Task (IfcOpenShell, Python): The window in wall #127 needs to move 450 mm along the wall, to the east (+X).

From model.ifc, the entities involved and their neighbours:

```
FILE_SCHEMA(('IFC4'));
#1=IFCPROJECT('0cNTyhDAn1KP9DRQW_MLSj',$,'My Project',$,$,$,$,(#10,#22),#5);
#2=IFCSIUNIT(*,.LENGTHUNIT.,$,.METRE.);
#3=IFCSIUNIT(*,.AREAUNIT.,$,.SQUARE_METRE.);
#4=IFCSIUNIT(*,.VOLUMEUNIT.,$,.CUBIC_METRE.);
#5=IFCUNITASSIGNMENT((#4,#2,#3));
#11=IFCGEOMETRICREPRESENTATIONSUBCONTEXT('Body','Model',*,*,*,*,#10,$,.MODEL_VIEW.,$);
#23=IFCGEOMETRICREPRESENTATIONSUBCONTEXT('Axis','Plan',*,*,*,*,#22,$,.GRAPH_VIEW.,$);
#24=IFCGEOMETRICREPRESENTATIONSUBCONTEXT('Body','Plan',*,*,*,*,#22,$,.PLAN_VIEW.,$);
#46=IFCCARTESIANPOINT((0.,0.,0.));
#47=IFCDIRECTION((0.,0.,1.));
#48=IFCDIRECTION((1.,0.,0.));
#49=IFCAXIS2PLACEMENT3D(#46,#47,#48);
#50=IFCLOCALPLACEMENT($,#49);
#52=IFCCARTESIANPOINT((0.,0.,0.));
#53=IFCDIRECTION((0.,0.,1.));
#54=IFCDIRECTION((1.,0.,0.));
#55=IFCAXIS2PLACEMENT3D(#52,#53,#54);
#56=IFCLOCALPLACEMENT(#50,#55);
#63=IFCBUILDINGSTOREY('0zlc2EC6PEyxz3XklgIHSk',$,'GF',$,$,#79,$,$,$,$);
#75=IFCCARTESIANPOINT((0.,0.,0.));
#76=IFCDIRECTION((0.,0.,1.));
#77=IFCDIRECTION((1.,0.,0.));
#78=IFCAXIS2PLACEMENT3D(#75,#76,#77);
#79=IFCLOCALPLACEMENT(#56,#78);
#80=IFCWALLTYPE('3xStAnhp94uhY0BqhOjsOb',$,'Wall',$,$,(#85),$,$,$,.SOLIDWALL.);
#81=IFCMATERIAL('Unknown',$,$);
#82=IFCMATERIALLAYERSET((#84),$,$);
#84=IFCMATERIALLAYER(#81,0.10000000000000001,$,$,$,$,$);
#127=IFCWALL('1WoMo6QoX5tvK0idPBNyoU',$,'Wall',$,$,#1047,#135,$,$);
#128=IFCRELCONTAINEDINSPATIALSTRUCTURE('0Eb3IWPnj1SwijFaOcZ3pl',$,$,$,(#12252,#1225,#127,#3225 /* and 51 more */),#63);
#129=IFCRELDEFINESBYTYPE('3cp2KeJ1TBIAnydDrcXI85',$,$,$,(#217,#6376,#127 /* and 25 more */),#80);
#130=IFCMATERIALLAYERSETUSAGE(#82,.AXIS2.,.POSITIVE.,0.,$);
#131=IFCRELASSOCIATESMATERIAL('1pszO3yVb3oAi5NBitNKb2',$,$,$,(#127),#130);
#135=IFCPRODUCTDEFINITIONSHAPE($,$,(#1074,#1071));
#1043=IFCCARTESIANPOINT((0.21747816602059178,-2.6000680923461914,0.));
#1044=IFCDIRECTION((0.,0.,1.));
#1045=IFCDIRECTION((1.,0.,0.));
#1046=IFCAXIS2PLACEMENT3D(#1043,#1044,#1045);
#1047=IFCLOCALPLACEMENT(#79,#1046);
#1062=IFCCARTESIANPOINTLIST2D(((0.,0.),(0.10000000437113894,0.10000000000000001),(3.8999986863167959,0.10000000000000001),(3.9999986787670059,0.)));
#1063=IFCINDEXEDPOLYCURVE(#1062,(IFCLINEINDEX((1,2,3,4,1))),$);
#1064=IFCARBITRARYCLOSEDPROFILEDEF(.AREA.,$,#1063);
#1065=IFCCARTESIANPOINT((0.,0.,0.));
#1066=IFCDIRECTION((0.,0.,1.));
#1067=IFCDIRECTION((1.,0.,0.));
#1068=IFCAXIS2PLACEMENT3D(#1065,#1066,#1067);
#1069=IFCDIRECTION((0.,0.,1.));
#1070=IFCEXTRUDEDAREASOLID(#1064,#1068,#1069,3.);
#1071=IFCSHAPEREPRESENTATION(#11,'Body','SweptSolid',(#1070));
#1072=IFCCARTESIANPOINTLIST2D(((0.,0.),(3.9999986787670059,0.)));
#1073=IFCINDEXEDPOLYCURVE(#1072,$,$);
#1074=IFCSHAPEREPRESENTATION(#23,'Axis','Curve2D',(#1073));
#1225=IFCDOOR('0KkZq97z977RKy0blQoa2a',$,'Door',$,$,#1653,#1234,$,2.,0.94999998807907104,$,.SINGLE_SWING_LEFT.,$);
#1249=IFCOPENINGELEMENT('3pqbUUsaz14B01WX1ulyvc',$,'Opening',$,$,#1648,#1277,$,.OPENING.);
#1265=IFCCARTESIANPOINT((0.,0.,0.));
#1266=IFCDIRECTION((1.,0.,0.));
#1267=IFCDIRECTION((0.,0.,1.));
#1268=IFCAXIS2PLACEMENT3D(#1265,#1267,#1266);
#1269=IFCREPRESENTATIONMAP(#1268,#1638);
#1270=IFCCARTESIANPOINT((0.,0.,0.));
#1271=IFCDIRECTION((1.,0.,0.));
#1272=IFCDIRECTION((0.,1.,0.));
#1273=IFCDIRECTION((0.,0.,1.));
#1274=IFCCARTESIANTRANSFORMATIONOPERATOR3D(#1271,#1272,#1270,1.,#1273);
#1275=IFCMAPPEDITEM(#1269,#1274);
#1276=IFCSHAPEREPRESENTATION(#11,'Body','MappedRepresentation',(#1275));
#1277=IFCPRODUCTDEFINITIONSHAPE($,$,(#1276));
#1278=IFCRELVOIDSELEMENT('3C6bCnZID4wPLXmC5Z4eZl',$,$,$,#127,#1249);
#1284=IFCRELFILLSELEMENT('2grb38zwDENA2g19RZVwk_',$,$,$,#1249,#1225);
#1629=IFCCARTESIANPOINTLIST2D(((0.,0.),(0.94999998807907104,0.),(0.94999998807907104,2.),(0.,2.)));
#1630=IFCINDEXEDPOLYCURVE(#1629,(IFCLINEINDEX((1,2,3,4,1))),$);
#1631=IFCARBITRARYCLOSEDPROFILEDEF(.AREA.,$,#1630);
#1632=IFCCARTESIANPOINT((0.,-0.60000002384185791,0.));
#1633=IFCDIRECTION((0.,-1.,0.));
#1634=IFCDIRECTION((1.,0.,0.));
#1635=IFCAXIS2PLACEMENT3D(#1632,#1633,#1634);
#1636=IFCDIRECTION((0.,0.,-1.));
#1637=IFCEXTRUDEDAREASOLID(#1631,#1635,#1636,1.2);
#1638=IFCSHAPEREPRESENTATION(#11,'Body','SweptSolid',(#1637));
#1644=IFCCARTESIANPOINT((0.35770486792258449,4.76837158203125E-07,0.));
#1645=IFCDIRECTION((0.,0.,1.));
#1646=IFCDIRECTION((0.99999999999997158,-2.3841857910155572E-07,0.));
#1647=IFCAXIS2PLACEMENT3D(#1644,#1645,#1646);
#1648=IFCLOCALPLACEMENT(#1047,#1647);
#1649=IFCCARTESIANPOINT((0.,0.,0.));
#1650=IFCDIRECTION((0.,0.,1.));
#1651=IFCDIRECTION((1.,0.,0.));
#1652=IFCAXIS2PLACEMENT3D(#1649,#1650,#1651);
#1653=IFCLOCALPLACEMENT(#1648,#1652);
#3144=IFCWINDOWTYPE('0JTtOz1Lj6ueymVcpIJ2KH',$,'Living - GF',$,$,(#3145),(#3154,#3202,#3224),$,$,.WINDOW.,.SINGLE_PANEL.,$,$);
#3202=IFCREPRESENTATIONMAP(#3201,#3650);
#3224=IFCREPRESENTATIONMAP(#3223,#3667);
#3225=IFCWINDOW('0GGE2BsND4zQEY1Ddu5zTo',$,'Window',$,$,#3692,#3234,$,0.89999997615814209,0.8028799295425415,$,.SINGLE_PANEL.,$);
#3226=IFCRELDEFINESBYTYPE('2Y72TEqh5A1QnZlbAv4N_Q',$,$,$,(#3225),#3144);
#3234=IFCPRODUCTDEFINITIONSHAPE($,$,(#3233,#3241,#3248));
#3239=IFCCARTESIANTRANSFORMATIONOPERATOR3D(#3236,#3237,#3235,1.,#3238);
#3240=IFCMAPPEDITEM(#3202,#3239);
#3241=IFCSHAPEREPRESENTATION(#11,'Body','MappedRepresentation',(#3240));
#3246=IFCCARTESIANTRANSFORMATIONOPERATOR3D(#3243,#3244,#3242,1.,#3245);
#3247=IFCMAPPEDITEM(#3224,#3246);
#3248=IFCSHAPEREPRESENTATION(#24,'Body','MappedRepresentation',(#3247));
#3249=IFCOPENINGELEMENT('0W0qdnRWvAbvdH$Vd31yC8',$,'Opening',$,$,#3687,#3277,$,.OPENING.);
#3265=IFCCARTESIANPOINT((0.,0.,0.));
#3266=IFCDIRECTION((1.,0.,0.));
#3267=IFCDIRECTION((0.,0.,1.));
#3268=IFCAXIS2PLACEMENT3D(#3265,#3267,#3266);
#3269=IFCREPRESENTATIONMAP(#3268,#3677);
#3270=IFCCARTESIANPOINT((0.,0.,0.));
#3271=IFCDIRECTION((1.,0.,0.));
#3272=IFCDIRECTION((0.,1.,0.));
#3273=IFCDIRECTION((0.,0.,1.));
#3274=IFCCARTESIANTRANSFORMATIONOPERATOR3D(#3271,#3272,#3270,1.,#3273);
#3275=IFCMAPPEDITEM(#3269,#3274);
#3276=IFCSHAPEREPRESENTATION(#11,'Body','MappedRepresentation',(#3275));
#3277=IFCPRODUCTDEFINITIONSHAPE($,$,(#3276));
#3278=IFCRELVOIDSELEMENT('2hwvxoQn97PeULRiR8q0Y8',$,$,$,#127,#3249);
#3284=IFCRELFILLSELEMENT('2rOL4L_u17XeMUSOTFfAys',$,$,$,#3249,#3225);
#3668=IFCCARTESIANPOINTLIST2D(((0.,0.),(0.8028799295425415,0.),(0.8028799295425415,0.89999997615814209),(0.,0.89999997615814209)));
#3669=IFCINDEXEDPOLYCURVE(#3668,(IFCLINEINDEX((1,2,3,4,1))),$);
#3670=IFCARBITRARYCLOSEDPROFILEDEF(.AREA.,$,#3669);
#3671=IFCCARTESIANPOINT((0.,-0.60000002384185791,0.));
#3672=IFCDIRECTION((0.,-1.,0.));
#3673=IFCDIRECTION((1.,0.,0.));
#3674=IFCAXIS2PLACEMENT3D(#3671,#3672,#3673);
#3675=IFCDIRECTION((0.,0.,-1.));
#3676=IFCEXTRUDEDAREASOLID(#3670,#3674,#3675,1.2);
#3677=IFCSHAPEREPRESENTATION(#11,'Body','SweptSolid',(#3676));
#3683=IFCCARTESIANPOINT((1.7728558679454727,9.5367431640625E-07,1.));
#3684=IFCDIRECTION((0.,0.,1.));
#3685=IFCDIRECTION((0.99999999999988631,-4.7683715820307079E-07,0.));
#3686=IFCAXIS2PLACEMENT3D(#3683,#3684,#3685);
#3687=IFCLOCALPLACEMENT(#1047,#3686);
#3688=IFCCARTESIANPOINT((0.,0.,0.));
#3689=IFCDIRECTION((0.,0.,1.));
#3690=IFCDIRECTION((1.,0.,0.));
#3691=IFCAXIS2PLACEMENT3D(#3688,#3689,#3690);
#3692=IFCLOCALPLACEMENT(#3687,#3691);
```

```python
import ifcopenshell
import ifcopenshell.api.geometry
import ifcopenshell.util.placement

model = ifcopenshell.open("model.ifc")

window = model.by_guid("0GGE2BsND4zQEY1Ddu5zTo")
opening = window.FillsVoids[0].RelatingOpeningElement
wall = opening.VoidsElements[0].RelatingBuildingElement

wall_matrix = ifcopenshell.util.placement.get_local_placement(wall.ObjectPlacement)
shift = wall_matrix[:3, 0] * 0.45
before = ifcopenshell.util.placement.get_local_placement(window.ObjectPlacement)[:3, 3].copy()

# The window is placed relative to its opening, so it follows when the opening moves.
matrix = ifcopenshell.util.placement.get_local_placement(opening.ObjectPlacement)
matrix[:3, 3] += shift
ifcopenshell.api.geometry.edit_object_placement(
    model, product=opening, matrix=matrix, is_si=False, should_transform_children=True
)

after = ifcopenshell.util.placement.get_local_placement(window.ObjectPlacement)[:3, 3]
print("window moved by", (after - before).round(3) + 0.0)

model.write("model_v2.ifc")
```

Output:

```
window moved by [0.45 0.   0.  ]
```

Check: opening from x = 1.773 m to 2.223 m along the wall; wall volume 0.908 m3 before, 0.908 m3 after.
